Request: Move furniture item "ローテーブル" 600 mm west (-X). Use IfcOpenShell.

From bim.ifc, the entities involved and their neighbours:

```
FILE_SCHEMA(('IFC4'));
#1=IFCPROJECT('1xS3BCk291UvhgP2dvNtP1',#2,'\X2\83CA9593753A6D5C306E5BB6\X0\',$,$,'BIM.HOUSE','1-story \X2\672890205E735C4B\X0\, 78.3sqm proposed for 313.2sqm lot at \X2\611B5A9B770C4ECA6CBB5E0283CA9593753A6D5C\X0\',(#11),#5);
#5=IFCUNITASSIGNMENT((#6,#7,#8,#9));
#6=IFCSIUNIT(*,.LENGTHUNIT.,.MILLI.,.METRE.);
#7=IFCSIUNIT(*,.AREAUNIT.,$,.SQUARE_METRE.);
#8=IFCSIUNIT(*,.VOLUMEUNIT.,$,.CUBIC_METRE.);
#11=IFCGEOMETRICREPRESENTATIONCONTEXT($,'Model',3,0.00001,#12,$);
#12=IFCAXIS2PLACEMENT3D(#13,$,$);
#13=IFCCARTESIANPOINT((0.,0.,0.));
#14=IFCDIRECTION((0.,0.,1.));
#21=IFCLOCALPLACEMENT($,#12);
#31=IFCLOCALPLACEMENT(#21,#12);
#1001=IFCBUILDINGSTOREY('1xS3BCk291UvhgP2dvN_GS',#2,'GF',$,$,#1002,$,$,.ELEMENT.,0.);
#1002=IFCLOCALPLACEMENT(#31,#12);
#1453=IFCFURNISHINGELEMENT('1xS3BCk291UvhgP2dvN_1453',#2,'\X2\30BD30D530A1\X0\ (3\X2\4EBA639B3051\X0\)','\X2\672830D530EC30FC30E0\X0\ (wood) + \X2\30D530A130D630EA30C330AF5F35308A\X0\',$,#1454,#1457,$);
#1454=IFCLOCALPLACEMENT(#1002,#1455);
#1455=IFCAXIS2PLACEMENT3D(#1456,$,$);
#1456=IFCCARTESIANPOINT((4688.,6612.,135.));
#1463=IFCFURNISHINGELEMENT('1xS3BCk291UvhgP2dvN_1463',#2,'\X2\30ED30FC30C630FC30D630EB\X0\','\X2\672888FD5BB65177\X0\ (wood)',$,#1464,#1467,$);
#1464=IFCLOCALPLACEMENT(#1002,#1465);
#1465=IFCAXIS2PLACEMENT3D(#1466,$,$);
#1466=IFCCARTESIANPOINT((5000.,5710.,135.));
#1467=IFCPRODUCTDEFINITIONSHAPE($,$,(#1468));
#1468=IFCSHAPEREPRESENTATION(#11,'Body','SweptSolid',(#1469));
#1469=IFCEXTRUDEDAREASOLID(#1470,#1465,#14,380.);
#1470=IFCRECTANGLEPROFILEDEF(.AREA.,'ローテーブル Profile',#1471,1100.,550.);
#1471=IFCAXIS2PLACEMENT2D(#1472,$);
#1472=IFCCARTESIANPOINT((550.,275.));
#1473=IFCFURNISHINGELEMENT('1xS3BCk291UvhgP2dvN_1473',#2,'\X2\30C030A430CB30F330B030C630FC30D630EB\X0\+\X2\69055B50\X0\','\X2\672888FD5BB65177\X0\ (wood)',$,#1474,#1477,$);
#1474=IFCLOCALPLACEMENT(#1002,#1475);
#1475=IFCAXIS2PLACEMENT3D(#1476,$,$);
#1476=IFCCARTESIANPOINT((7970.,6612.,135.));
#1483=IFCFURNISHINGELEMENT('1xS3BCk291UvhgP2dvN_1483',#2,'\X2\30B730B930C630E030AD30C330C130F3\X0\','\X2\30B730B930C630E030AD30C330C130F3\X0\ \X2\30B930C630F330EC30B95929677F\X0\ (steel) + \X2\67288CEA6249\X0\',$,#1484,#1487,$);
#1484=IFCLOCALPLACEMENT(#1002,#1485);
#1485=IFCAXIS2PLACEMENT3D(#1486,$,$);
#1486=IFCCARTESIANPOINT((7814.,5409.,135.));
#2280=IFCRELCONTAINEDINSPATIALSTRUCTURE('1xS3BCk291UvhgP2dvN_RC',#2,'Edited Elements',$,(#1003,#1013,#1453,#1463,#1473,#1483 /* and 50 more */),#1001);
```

```python
import ifcopenshell
import ifcopenshell.api.geometry
import ifcopenshell.util.placement

model = ifcopenshell.open("bim.ifc")

item = model.by_id(1463)
matrix = ifcopenshell.util.placement.get_local_placement(item.ObjectPlacement)
matrix[0, 3] -= 600.0
ifcopenshell.api.geometry.edit_object_placement(model, product=item, matrix=matrix, is_si=False)

print(ifcopenshell.util.placement.get_local_placement(item.ObjectPlacement).round(3) + 0.0)

model.write("bim_rev.ifc")
```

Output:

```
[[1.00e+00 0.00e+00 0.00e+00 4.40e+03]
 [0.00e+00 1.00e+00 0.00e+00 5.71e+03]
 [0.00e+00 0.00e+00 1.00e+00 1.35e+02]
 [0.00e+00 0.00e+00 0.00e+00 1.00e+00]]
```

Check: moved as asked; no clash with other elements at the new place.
